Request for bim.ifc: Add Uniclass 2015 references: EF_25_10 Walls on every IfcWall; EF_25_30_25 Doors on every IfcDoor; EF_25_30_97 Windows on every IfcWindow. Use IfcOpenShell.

First a look at what the model holds.

```python
import ifcopenshell

model = ifcopenshell.open("bim.ifc")
print(model.schema)
print("classifications:", [c.Name for c in model.by_type("IfcClassification")])
for ifc_class in ("IfcDoor", "IfcRoof", "IfcStair", "IfcWall", "IfcWindow"):
    print(ifc_class, len(model.by_type(ifc_class)))
```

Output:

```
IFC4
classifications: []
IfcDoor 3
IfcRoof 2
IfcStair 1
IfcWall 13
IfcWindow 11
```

```python
import ifcopenshell
import ifcopenshell.api.classification

model = ifcopenshell.open("bim.ifc")

system = ifcopenshell.api.classification.add_classification(model, classification="Uniclass 2015")

codes = {
    "IfcWall": ("EF_25_10", "Walls"),
    "IfcDoor": ("EF_25_30_25", "Doors"),
    "IfcWindow": ("EF_25_30_97", "Windows"),
}
for ifc_class, (code, name) in codes.items():
    products = model.by_type(ifc_class)
    ifcopenshell.api.classification.add_reference(
        model, products=products, classification=system, identification=code, name=name
    )
    print(code, len(products))

model.write("bim-out.ifc")
```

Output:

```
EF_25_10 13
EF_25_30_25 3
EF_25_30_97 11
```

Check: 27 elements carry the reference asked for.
